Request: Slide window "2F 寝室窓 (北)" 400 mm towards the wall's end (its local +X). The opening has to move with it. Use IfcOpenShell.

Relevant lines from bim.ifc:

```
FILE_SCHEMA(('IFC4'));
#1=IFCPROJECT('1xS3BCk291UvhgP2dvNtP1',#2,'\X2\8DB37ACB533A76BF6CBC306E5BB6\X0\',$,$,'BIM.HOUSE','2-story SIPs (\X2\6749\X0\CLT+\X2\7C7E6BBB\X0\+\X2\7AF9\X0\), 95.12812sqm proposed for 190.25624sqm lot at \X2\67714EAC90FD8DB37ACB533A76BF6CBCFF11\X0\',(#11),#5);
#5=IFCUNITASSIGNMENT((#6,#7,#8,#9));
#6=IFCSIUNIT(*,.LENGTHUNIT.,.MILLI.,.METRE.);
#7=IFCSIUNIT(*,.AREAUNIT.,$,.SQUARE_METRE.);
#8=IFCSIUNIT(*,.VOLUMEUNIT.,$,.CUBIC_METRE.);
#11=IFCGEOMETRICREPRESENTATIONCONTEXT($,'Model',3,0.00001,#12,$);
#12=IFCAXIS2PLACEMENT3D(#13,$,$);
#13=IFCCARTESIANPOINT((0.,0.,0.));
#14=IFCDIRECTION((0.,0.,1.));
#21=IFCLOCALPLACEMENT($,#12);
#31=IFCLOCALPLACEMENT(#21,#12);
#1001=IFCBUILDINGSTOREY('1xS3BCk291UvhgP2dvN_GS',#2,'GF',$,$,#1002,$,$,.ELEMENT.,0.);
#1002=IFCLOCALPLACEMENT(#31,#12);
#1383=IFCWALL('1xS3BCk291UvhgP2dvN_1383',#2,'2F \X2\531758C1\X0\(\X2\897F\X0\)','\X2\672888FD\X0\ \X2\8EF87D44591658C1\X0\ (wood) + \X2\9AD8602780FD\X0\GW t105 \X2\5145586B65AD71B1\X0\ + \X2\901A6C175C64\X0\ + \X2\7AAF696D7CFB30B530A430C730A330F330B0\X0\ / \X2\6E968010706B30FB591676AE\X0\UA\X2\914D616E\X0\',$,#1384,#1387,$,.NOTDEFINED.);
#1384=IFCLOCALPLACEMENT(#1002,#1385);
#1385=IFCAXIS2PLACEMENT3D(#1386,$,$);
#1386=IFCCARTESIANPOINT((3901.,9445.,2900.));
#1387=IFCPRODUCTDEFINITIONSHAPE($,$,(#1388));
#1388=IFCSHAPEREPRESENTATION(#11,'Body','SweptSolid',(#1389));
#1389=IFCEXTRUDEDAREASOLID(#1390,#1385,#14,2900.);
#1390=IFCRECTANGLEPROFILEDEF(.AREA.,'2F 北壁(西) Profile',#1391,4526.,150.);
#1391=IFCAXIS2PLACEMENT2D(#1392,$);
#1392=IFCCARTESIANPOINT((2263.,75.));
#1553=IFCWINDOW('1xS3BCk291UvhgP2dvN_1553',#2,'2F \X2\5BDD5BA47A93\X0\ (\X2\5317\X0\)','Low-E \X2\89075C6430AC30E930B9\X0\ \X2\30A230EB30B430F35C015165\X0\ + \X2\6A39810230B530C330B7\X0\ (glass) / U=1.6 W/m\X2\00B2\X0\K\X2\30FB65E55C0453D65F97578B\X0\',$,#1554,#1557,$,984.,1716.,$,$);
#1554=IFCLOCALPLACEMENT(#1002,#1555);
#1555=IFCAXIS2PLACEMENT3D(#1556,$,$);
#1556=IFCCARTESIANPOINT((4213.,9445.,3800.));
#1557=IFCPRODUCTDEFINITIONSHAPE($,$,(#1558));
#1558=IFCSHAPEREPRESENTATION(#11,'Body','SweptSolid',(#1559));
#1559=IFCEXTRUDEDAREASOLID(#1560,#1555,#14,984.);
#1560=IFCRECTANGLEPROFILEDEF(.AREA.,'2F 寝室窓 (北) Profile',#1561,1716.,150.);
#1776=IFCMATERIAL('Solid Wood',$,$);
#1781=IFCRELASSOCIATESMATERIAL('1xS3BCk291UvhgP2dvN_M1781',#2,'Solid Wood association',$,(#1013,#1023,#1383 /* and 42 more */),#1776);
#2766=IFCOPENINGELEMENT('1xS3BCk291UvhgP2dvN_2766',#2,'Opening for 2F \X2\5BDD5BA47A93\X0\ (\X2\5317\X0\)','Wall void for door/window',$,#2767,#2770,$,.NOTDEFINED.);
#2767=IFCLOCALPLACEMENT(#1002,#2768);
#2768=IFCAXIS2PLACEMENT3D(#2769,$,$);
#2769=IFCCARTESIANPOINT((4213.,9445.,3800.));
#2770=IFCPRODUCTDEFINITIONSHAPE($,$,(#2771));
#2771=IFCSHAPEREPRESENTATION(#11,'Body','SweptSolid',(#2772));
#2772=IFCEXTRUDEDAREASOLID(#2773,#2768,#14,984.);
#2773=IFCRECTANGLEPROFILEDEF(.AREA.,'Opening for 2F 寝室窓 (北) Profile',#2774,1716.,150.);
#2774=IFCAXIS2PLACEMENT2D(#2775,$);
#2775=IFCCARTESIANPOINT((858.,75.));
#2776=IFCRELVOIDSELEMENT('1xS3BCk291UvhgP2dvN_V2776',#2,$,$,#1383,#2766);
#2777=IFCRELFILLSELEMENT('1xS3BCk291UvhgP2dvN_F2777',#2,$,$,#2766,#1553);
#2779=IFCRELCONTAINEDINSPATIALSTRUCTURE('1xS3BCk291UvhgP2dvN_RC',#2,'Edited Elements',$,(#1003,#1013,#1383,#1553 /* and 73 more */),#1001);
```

```python
import ifcopenshell
import ifcopenshell.api.geometry
import ifcopenshell.util.placement
import ifcopenshell.util.unit

model = ifcopenshell.open("bim.ifc")
unit_scale = ifcopenshell.util.unit.calculate_unit_scale(model)

window = model.by_guid("1xS3BCk291UvhgP2dvN_1553")
opening = window.FillsVoids[0].RelatingOpeningElement
wall = opening.VoidsElements[0].RelatingBuildingElement

wall_matrix = ifcopenshell.util.placement.get_local_placement(wall.ObjectPlacement)
shift = wall_matrix[:3, 0] * 0.4 / unit_scale
before = ifcopenshell.util.placement.get_local_placement(window.ObjectPlacement)[:3, 3].copy()

# The window is not placed relative to its opening, so move both.
for product in (opening, window):
    matrix = ifcopenshell.util.placement.get_local_placement(product.ObjectPlacement)
    matrix[:3, 3] += shift
    ifcopenshell.api.geometry.edit_object_placement(model, product=product, matrix=matrix, is_si=False)

after = ifcopenshell.util.placement.get_local_placement(window.ObjectPlacement)[:3, 3]
print("window moved by", (after - before).round(3) + 0.0)

model.write("bim_rev.ifc")
```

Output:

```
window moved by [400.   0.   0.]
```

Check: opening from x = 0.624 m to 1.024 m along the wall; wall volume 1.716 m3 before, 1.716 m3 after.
